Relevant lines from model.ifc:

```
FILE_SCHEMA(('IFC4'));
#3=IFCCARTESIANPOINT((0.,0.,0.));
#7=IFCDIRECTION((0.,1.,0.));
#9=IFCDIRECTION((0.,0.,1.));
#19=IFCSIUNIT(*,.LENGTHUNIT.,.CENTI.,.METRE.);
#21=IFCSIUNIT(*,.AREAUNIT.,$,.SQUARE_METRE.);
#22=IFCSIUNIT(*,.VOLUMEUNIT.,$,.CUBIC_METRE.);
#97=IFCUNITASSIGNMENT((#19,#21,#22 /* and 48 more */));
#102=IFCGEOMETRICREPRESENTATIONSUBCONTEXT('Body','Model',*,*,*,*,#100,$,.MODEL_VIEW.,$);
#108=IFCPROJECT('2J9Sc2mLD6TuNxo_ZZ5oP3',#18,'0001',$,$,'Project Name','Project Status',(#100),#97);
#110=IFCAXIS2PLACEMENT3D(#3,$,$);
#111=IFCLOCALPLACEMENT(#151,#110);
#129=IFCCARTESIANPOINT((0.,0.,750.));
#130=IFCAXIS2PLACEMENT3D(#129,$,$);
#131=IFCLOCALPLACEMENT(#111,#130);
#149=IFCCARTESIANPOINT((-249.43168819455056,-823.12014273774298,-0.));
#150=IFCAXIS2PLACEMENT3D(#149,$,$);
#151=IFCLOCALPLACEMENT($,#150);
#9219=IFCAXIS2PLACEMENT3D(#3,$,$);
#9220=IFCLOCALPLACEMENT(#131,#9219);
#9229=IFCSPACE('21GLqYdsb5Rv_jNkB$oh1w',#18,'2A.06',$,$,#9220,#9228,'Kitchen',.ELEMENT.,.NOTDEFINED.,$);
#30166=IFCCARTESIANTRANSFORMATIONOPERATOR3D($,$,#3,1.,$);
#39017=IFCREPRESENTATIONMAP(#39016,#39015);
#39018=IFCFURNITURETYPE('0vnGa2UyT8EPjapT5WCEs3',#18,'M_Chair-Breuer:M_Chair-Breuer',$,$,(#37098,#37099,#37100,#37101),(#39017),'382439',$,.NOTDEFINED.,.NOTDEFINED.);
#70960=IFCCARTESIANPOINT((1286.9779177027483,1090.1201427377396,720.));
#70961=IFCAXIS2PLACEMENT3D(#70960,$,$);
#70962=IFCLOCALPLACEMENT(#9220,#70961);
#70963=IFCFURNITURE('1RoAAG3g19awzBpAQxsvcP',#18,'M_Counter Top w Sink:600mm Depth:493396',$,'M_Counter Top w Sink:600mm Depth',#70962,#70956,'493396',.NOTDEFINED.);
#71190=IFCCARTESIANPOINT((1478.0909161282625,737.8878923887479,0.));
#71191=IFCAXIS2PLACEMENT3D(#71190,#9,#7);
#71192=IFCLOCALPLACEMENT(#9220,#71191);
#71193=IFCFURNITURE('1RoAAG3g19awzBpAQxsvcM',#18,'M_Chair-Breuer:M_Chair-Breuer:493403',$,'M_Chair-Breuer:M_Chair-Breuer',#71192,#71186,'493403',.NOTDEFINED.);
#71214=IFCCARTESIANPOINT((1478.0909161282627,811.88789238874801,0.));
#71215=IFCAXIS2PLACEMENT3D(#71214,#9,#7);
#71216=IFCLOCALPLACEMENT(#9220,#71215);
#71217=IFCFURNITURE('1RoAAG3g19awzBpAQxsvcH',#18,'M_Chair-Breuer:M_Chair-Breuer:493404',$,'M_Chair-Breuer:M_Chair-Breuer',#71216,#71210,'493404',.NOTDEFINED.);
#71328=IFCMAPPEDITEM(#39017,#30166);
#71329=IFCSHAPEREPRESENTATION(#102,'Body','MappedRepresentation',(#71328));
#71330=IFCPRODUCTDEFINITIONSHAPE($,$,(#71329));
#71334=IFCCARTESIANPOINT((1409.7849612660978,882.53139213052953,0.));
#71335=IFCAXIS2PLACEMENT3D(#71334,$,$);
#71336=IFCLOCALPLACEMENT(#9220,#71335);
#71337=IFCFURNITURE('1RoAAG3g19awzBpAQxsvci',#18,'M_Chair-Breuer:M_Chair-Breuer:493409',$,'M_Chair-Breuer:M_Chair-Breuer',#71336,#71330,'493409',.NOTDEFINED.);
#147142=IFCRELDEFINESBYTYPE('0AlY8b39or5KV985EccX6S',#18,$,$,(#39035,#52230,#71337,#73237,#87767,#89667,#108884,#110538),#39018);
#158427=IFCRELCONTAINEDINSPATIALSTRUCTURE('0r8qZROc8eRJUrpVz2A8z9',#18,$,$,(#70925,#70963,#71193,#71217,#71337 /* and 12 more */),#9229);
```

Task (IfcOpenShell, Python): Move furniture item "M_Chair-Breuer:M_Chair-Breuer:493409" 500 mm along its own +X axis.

```python
import ifcopenshell
import ifcopenshell.api.geometry
import ifcopenshell.util.placement
import ifcopenshell.util.unit

model = ifcopenshell.open("model.ifc")
unit_scale = ifcopenshell.util.unit.calculate_unit_scale(model)

item = model.by_id(71337)
matrix = ifcopenshell.util.placement.get_local_placement(item.ObjectPlacement)
matrix[:3, 3] += matrix[:3, 0] * 0.5 / unit_scale
ifcopenshell.api.geometry.edit_object_placement(model, product=item, matrix=matrix, is_si=False)

print(ifcopenshell.util.placement.get_local_placement(item.ObjectPlacement).round(3) + 0.0)

model.write("model_rev.ifc")
```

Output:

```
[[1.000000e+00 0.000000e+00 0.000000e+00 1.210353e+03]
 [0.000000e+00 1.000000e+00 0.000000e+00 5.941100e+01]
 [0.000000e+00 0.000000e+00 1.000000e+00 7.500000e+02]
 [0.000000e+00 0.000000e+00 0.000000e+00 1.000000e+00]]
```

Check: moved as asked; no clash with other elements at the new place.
